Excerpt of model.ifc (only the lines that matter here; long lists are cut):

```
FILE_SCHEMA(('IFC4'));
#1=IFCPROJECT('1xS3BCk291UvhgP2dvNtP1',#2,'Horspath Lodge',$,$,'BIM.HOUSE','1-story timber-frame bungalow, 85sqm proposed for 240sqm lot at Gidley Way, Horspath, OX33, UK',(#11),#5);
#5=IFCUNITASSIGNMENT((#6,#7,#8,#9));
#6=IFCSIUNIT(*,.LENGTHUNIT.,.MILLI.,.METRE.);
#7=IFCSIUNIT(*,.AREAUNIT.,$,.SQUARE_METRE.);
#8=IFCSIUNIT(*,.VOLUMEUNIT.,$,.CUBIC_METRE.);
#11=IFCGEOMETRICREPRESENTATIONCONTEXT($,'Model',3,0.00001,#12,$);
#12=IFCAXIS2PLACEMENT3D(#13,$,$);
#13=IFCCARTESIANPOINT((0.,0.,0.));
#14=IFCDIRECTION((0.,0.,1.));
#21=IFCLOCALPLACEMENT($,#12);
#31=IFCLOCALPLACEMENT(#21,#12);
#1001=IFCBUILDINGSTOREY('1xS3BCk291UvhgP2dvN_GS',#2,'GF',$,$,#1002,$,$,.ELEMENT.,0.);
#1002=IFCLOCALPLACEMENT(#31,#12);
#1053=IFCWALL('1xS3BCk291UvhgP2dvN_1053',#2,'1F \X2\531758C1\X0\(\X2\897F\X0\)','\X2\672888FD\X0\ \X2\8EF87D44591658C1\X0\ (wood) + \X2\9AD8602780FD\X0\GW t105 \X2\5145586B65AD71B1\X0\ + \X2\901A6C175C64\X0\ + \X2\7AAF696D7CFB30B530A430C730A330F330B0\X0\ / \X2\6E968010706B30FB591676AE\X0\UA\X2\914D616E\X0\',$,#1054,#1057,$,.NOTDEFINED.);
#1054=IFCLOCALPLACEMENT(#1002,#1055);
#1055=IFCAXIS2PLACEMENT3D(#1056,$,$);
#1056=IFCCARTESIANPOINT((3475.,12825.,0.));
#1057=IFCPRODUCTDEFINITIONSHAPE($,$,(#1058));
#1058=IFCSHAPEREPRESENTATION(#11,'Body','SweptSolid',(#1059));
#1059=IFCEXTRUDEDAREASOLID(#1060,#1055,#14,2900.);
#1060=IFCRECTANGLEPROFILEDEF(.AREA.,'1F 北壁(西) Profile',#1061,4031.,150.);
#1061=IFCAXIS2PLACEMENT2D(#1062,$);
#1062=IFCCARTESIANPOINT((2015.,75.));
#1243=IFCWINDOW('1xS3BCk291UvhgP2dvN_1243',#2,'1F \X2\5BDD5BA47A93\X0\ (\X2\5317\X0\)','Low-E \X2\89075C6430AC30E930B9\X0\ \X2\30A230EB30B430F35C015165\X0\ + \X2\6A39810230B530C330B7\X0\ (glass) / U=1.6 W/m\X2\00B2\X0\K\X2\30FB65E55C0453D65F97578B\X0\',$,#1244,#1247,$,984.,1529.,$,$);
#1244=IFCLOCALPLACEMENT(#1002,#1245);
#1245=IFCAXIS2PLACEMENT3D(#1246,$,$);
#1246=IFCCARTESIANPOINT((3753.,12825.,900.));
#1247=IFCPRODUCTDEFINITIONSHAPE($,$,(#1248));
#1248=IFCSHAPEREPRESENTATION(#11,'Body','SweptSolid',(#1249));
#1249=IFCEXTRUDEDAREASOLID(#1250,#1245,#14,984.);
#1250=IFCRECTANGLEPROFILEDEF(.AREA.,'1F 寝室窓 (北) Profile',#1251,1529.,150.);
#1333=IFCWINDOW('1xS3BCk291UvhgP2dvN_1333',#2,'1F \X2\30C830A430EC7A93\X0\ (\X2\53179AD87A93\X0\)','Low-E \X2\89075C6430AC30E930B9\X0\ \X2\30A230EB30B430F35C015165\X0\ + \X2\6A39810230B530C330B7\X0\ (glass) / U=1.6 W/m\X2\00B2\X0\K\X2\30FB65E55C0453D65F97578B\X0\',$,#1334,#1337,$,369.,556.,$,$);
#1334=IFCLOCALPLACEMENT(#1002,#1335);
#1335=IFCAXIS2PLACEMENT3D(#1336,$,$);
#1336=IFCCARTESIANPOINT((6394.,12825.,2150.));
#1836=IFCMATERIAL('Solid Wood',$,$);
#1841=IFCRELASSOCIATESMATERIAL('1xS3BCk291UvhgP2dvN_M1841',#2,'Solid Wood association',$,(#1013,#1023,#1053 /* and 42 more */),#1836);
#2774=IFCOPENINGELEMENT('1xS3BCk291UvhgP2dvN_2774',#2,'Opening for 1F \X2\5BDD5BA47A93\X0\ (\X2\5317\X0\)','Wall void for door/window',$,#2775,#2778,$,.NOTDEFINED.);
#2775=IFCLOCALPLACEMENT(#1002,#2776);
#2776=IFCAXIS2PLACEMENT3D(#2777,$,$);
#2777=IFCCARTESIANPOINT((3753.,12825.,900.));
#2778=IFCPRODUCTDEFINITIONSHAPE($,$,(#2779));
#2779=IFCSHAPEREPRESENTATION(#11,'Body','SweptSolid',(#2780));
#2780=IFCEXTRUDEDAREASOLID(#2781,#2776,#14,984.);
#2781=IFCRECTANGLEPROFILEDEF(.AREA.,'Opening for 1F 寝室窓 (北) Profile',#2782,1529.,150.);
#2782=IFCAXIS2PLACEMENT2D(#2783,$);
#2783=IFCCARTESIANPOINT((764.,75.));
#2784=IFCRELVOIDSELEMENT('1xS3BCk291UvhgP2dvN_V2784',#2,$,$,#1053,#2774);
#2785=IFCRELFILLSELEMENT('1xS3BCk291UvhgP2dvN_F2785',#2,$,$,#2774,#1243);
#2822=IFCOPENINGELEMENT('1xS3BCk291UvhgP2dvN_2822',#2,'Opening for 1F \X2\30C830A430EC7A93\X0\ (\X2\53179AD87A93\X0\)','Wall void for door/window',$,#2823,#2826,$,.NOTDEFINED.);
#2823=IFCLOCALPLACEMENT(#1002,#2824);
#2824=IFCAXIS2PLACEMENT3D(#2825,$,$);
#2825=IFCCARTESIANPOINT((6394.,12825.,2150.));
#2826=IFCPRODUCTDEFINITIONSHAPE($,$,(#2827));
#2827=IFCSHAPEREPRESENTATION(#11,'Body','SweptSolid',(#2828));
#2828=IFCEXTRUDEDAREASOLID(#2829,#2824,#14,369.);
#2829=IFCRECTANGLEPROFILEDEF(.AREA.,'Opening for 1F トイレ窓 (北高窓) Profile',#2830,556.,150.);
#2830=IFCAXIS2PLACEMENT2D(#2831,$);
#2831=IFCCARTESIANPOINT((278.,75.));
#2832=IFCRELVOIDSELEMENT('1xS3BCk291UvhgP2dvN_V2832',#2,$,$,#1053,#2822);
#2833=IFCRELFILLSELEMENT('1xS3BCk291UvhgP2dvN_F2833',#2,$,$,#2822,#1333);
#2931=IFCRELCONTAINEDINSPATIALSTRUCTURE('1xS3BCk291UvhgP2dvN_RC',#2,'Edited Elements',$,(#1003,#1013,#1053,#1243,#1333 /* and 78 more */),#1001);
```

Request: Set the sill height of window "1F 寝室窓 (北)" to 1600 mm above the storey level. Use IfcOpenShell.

```python
import numpy as np
import ifcopenshell
import ifcopenshell.api.geometry
import ifcopenshell.geom
import ifcopenshell.util.element
import ifcopenshell.util.placement
import ifcopenshell.util.shape
import ifcopenshell.util.unit

model = ifcopenshell.open("model.ifc")
unit_scale = ifcopenshell.util.unit.calculate_unit_scale(model)

window = model.by_guid("1xS3BCk291UvhgP2dvN_1243")
opening = window.FillsVoids[0].RelatingOpeningElement
storey = ifcopenshell.util.element.get_container(window, ifc_class="IfcBuildingStorey")
level = ifcopenshell.util.placement.get_local_placement(storey.ObjectPlacement)[2, 3]

# The opening's origin need not be at the sill, so measure its lowest point.
shape = ifcopenshell.geom.create_shape(ifcopenshell.geom.settings(), opening)
bottom = ifcopenshell.util.shape.get_shape_bottom_elevation(shape, shape.geometry) / unit_scale
dz = level + 1.6 / unit_scale - bottom

shift = np.array([0.0, 0.0, dz])
# The window is not placed relative to its opening, so move both.
for product in (opening, window):
    matrix = ifcopenshell.util.placement.get_local_placement(product.ObjectPlacement)
    matrix[:3, 3] += shift
    ifcopenshell.api.geometry.edit_object_placement(model, product=product, matrix=matrix, is_si=False)

print(f"moved by {dz * unit_scale:+.3f} m")

model.write("model-out.ifc")
```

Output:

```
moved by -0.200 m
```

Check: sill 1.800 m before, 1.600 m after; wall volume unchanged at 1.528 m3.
